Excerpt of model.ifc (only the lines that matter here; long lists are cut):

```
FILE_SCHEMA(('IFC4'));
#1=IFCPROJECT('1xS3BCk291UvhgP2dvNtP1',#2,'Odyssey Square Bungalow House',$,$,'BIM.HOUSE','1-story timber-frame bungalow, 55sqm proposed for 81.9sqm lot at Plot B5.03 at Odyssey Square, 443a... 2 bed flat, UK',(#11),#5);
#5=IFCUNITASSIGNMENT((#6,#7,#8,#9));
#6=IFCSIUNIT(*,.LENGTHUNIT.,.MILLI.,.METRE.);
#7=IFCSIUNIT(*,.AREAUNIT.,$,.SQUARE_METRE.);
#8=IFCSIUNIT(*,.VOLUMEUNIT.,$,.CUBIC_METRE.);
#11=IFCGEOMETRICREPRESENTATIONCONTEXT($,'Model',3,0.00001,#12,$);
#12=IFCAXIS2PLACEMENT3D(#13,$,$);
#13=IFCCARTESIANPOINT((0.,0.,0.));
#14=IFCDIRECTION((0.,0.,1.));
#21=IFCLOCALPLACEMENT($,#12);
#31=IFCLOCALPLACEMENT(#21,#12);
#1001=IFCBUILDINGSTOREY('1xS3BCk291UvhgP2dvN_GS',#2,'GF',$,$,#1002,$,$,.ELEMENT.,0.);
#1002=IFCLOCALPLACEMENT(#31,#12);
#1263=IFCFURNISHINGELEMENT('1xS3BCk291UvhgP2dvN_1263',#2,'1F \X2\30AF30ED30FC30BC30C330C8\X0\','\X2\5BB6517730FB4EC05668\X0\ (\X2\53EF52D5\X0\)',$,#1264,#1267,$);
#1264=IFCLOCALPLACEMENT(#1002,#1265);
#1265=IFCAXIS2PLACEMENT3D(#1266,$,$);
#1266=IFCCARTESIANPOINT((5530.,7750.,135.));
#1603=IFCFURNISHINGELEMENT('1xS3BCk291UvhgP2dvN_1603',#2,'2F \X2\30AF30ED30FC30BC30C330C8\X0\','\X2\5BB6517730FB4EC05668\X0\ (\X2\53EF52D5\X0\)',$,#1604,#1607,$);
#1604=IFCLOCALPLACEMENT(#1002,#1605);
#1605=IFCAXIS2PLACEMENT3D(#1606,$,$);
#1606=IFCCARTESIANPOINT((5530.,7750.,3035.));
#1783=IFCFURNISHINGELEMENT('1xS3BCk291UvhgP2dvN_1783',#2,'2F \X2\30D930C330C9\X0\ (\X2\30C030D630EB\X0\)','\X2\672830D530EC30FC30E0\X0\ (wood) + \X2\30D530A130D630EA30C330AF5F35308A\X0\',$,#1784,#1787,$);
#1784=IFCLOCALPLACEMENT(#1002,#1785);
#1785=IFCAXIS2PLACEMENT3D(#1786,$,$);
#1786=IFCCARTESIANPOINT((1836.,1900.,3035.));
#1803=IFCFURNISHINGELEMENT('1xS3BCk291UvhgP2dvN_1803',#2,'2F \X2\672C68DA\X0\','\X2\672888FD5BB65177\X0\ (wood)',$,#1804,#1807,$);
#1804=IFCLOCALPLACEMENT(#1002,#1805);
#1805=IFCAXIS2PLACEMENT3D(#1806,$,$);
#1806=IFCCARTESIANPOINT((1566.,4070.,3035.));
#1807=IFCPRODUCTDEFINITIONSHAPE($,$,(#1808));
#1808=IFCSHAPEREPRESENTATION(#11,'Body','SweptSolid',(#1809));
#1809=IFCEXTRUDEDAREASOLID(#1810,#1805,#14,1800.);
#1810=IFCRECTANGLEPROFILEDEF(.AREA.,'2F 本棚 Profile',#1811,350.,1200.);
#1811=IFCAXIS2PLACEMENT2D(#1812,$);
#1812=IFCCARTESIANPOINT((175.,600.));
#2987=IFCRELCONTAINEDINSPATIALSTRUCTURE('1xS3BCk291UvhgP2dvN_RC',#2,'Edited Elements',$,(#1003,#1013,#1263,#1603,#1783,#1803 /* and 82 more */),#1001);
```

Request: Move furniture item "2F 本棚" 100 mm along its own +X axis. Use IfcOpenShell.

```python
import ifcopenshell
import ifcopenshell.api.geometry
import ifcopenshell.util.placement
import ifcopenshell.util.unit

model = ifcopenshell.open("model.ifc")
unit_scale = ifcopenshell.util.unit.calculate_unit_scale(model)

item = model.by_guid("1xS3BCk291UvhgP2dvN_1803")
matrix = ifcopenshell.util.placement.get_local_placement(item.ObjectPlacement)
matrix[:3, 3] += matrix[:3, 0] * 0.1 / unit_scale
ifcopenshell.api.geometry.edit_object_placement(model, product=item, matrix=matrix, is_si=False)

print(ifcopenshell.util.placement.get_local_placement(item.ObjectPlacement).round(3) + 0.0)

model.write("model_v2.ifc")
```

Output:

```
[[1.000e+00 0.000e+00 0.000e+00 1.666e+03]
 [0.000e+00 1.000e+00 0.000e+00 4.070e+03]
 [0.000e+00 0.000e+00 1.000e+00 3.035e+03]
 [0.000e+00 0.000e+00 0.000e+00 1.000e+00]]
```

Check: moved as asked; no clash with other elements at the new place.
